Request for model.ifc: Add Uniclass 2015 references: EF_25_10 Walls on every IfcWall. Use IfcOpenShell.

First a look at what the model holds.

```python
import ifcopenshell

model = ifcopenshell.open("model.ifc")
print(model.schema)
print("classifications:", [c.Name for c in model.by_type("IfcClassification")])
for ifc_class in ("IfcDoor", "IfcRoof", "IfcStair", "IfcWall", "IfcWindow"):
    print(ifc_class, len(model.by_type(ifc_class)))
```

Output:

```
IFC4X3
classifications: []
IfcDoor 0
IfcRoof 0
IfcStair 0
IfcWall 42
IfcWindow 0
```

```python
import ifcopenshell
import ifcopenshell.api.classification

model = ifcopenshell.open("model.ifc")

system = ifcopenshell.api.classification.add_classification(model, classification="Uniclass 2015")

codes = {
    "IfcWall": ("EF_25_10", "Walls"),
}
for ifc_class, (code, name) in codes.items():
    products = model.by_type(ifc_class)
    ifcopenshell.api.classification.add_reference(
        model, products=products, classification=system, identification=code, name=name
    )
    print(code, len(products))

model.write("model_v2.ifc")
```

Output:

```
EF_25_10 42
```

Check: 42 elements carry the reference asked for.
